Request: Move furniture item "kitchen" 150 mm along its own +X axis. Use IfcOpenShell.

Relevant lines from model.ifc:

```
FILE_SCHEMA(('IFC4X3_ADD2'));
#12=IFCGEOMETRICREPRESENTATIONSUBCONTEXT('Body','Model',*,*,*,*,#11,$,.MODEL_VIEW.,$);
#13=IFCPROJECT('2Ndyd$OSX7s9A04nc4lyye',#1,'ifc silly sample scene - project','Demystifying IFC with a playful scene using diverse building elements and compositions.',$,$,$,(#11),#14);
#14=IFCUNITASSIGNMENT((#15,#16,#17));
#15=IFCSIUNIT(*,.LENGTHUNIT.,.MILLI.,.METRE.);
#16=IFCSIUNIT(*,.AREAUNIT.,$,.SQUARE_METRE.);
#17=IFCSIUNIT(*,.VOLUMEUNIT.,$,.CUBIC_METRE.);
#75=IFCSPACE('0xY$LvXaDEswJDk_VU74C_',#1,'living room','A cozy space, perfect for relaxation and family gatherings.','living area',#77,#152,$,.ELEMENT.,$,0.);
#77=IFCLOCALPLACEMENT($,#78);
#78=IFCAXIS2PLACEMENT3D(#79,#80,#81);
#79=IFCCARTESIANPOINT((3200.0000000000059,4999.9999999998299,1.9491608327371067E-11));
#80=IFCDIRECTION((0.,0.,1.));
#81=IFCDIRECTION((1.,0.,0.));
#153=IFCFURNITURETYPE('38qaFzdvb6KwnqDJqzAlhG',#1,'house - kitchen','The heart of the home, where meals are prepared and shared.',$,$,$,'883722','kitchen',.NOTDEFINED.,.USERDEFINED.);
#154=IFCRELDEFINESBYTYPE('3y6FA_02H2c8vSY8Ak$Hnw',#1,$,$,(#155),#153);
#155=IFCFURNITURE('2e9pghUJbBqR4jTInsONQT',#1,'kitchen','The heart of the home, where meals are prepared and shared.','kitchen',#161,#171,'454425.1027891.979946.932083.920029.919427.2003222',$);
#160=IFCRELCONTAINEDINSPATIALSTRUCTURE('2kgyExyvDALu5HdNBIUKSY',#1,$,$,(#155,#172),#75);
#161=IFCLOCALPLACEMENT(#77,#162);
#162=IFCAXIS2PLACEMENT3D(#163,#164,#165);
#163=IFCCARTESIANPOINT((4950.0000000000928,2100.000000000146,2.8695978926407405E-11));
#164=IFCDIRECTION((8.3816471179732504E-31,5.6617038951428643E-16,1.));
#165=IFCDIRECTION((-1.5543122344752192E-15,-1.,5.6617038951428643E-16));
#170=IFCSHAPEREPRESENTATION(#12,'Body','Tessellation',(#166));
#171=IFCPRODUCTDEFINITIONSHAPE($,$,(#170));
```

```python
import ifcopenshell
import ifcopenshell.api.geometry
import ifcopenshell.util.placement

model = ifcopenshell.open("model.ifc")

item = model.by_guid("2e9pghUJbBqR4jTInsONQT")
matrix = ifcopenshell.util.placement.get_local_placement(item.ObjectPlacement)
matrix[:3, 3] += matrix[:3, 0] * 150.0
ifcopenshell.api.geometry.edit_object_placement(model, product=item, matrix=matrix, is_si=False)

print(ifcopenshell.util.placement.get_local_placement(item.ObjectPlacement).round(3) + 0.0)

model.write("model_edited.ifc")
```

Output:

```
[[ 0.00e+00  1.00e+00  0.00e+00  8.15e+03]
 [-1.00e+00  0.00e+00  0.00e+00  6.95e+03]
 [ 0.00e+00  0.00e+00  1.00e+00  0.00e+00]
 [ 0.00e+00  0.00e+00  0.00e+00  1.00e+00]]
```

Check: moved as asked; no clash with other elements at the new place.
